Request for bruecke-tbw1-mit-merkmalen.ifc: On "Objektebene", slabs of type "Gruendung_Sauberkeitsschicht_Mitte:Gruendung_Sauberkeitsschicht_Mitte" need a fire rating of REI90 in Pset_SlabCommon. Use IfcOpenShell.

First a look at what the model holds.

```python
import ifcopenshell
import ifcopenshell.util.element

model = ifcopenshell.open("bruecke-tbw1-mit-merkmalen.ifc")
print(model.schema)
storey = next(s for s in model.by_type("IfcBuildingStorey") if s.Name == "Objektebene")
slabs = [e for e in ifcopenshell.util.element.get_decomposition(storey) if e.is_a("IfcSlab")]
seen = {}
for e in slabs:
    element_type = ifcopenshell.util.element.get_type(e)
    key = (element_type.Name if element_type != e and element_type else None, ifcopenshell.util.element.get_pset(e, "Pset_SlabCommon", "FireRating"))
    seen[key] = seen.get(key, 0) + 1
for (name, value), count in sorted(seen.items(), key=str):
    print(count, "x", name, "|", value)
```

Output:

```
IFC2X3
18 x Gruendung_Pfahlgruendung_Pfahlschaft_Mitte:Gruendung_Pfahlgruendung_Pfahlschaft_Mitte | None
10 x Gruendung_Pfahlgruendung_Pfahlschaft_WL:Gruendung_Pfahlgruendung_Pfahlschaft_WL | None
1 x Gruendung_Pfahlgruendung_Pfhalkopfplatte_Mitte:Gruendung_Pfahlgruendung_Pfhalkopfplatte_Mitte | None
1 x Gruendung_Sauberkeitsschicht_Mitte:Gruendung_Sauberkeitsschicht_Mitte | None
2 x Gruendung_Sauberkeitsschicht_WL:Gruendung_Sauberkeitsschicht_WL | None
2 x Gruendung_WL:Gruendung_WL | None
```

```python
import ifcopenshell
import ifcopenshell.api.pset
import ifcopenshell.util.element

model = ifcopenshell.open("bruecke-tbw1-mit-merkmalen.ifc")

storey = next(s for s in model.by_type("IfcBuildingStorey") if s.Name == "Objektebene")
slabs = [e for e in ifcopenshell.util.element.get_decomposition(storey) if e.is_a("IfcSlab")]

count = 0
for e in slabs:
    element_type = ifcopenshell.util.element.get_type(e)
    if element_type in (None, e) or element_type.Name != "Gruendung_Sauberkeitsschicht_Mitte:Gruendung_Sauberkeitsschicht_Mitte":
        continue
    # add_pset returns the element's existing set when there is one.
    pset = ifcopenshell.api.pset.add_pset(model, product=e, name="Pset_SlabCommon")
    ifcopenshell.api.pset.edit_pset(model, pset=pset, properties={"FireRating": "REI90"})
    count += 1

print(count, "slabs updated")

model.write("bruecke-tbw1-mit-merkmalen-out.ifc")
```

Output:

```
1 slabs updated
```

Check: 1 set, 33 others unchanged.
